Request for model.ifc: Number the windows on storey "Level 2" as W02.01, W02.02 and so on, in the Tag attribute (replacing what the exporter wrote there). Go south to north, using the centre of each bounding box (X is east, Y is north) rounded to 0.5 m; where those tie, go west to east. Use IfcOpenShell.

First a look at what the model holds.

```python
import ifcopenshell
import ifcopenshell.util.element
import ifcopenshell.util.placement

model = ifcopenshell.open("model.ifc")
print(model.schema)
storey = next(s for s in model.by_type("IfcBuildingStorey") if s.Name == "Level 2")
windows = [e for e in ifcopenshell.util.element.get_decomposition(storey) if e.is_a("IfcWindow")]
for e in sorted(windows, key=lambda e: e.id()):
    origin = ifcopenshell.util.placement.get_local_placement(e.ObjectPlacement)[:3, 3]
    print(e.id(), e.Tag, e.Name, origin.round(2) + 0.0, sep=" | ")
```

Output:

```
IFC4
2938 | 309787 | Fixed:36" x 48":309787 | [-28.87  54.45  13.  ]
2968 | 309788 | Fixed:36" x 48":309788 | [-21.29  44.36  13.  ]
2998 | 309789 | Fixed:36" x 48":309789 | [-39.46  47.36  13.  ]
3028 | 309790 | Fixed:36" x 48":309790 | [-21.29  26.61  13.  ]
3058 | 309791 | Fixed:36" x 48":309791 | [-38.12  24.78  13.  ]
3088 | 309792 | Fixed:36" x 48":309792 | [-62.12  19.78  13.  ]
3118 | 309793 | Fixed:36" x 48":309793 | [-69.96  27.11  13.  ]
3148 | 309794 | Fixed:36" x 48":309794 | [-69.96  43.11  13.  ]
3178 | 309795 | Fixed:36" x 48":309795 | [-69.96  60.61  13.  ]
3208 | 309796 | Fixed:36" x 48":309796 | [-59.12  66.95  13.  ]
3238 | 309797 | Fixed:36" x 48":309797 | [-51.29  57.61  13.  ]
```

```python
import ifcopenshell
import ifcopenshell.geom
import ifcopenshell.util.element
import ifcopenshell.util.shape

model = ifcopenshell.open("model.ifc")
settings = ifcopenshell.geom.settings()
settings.set("use-world-coords", True)


def centre(element):
    shape = ifcopenshell.geom.create_shape(settings, element)
    return ifcopenshell.util.shape.get_bbox_centroid(shape.geometry)


storey = next(s for s in model.by_type("IfcBuildingStorey") if s.Name == "Level 2")
windows = [e for e in ifcopenshell.util.element.get_decomposition(storey) if e.is_a("IfcWindow")]

# Insertion points can sit at a corner or the storey origin, so sort by the geometry (in metres).
centres = {e: centre(e) for e in windows}
windows.sort(key=lambda e: (round(centres[e][1] / 0.5), centres[e][0]))

for i, e in enumerate(windows, start=1):
    number = f"W02.{i:02d}"
    e.Tag = number
    print(e.id(), number)

model.write("model_rev.ifc")
```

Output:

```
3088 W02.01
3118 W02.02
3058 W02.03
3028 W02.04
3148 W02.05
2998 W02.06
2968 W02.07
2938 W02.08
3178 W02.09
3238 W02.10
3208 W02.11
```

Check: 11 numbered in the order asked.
